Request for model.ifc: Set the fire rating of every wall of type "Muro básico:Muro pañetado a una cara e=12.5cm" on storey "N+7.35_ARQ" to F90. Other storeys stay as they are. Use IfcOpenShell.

First a look at what the model holds.

```python
import ifcopenshell
import ifcopenshell.util.element

model = ifcopenshell.open("model.ifc")
print(model.schema)
storey = next(s for s in model.by_type("IfcBuildingStorey") if s.Name == "N+7.35_ARQ")
walls = [e for e in ifcopenshell.util.element.get_decomposition(storey) if e.is_a("IfcWall")]
seen = {}
for e in walls:
    element_type = ifcopenshell.util.element.get_type(e)
    key = (element_type.Name if element_type != e and element_type else None, ifcopenshell.util.element.get_pset(e, "Pset_WallCommon", "FireRating"))
    seen[key] = seen.get(key, 0) + 1
for (name, value), count in sorted(seen.items(), key=str):
    print(count, "x", name, "|", value)
```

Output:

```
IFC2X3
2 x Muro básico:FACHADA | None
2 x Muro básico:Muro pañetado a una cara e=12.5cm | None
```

```python
import ifcopenshell
import ifcopenshell.api.pset
import ifcopenshell.util.element

model = ifcopenshell.open("model.ifc")

storey = next(s for s in model.by_type("IfcBuildingStorey") if s.Name == "N+7.35_ARQ")
walls = [e for e in ifcopenshell.util.element.get_decomposition(storey) if e.is_a("IfcWall")]

count = 0
for e in walls:
    element_type = ifcopenshell.util.element.get_type(e)
    if element_type in (None, e) or element_type.Name != "Muro básico:Muro pañetado a una cara e=12.5cm":
        continue
    # add_pset returns the element's existing set when there is one.
    pset = ifcopenshell.api.pset.add_pset(model, product=e, name="Pset_WallCommon")
    ifcopenshell.api.pset.edit_pset(model, pset=pset, properties={"FireRating": "F90"})
    count += 1

print(count, "walls updated")

model.write("model_edited.ifc")
```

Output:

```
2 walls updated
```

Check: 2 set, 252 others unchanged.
